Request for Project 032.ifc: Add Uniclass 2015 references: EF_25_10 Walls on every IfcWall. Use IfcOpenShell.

First a look at what the model holds.

```python
import ifcopenshell

model = ifcopenshell.open("Project 032.ifc")
print(model.schema)
print("classifications:", [c.Name for c in model.by_type("IfcClassification")])
for ifc_class in ("IfcDoor", "IfcRoof", "IfcStair", "IfcWall", "IfcWindow"):
    print(ifc_class, len(model.by_type(ifc_class)))
```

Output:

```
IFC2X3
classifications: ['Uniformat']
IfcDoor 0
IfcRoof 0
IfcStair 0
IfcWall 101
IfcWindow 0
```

```python
import ifcopenshell
import ifcopenshell.api.classification

model = ifcopenshell.open("Project 032.ifc")

# IFC2X3 requires Source and Edition and has no link from the project to the system.
system = model.create_entity("IfcClassification", Source="NBS", Edition="2015", Name="Uniclass 2015")

codes = {
    "IfcWall": ("EF_25_10", "Walls"),
}
for ifc_class, (code, name) in codes.items():
    products = model.by_type(ifc_class)
    ifcopenshell.api.classification.add_reference(
        model, products=products, classification=system, identification=code, name=name
    )
    print(code, len(products))

model.write("Project 032_updated.ifc")
```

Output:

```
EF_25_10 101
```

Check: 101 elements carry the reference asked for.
